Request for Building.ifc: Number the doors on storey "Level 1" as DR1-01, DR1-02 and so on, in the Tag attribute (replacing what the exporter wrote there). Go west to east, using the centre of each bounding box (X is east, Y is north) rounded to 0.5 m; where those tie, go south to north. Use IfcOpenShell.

First a look at what the model holds.

```python
import ifcopenshell
import ifcopenshell.util.element
import ifcopenshell.util.placement

model = ifcopenshell.open("Building.ifc")
print(model.schema)
storey = next(s for s in model.by_type("IfcBuildingStorey") if s.Name == "Level 1")
doors = [e for e in ifcopenshell.util.element.get_decomposition(storey) if e.is_a("IfcDoor")]
for e in sorted(doors, key=lambda e: e.id()):
    origin = ifcopenshell.util.placement.get_local_placement(e.ObjectPlacement)[:3, 3]
    print(e.id(), e.Tag, e.Name, origin.round(2) + 0.0, sep=" | ")
```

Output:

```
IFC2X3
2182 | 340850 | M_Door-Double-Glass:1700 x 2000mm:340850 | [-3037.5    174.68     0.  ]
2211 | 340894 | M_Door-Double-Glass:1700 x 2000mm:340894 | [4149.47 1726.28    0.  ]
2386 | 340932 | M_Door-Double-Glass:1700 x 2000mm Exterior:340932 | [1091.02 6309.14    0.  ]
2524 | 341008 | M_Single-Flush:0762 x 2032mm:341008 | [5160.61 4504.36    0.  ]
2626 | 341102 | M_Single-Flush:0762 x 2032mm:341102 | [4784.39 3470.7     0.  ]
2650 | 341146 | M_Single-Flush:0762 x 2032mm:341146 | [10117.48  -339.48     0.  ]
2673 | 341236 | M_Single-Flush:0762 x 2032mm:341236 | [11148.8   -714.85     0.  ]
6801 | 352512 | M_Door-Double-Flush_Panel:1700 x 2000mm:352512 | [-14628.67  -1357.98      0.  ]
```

```python
import ifcopenshell
import ifcopenshell.geom
import ifcopenshell.util.element
import ifcopenshell.util.shape

model = ifcopenshell.open("Building.ifc")
settings = ifcopenshell.geom.settings()
settings.set("use-world-coords", True)


def centre(element):
    shape = ifcopenshell.geom.create_shape(settings, element)
    return ifcopenshell.util.shape.get_bbox_centroid(shape.geometry)


storey = next(s for s in model.by_type("IfcBuildingStorey") if s.Name == "Level 1")
doors = [e for e in ifcopenshell.util.element.get_decomposition(storey) if e.is_a("IfcDoor")]

# Insertion points can sit at a corner or the storey origin, so sort by the geometry (in metres).
centres = {e: centre(e) for e in doors}
doors.sort(key=lambda e: (round(centres[e][0] / 0.5), centres[e][1]))

for i, e in enumerate(doors, start=1):
    number = f"DR1-{i:02d}"
    e.Tag = number
    print(e.id(), number)

model.write("Building_updated.ifc")
```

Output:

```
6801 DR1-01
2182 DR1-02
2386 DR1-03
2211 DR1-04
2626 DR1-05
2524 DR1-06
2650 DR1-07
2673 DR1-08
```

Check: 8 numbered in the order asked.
